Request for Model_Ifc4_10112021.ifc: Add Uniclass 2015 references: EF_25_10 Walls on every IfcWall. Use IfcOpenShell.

First a look at what the model holds.

```python
import ifcopenshell

model = ifcopenshell.open("Model_Ifc4_10112021.ifc")
print(model.schema)
print("classifications:", [c.Name for c in model.by_type("IfcClassification")])
for ifc_class in ("IfcDoor", "IfcRoof", "IfcStair", "IfcWall", "IfcWindow"):
    print(ifc_class, len(model.by_type(ifc_class)))
```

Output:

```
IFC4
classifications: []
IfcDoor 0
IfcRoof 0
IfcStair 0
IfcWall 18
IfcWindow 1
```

```python
import ifcopenshell
import ifcopenshell.api.classification

model = ifcopenshell.open("Model_Ifc4_10112021.ifc")

system = ifcopenshell.api.classification.add_classification(model, classification="Uniclass 2015")

codes = {
    "IfcWall": ("EF_25_10", "Walls"),
}
for ifc_class, (code, name) in codes.items():
    products = model.by_type(ifc_class)
    ifcopenshell.api.classification.add_reference(
        model, products=products, classification=system, identification=code, name=name
    )
    print(code, len(products))

model.write("Model_Ifc4_10112021_edited.ifc")
```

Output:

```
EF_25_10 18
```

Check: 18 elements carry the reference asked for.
